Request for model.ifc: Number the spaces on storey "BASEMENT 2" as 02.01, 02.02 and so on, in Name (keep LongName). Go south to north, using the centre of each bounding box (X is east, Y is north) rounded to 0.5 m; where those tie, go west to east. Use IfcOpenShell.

First a look at what the model holds.

```python
import ifcopenshell
import ifcopenshell.util.element
import ifcopenshell.util.placement

model = ifcopenshell.open("model.ifc")
print(model.schema)
storey = next(s for s in model.by_type("IfcBuildingStorey") if s.Name == "BASEMENT 2")
spaces = [e for e in ifcopenshell.util.element.get_decomposition(storey) if e.is_a("IfcSpace")]
for e in sorted(spaces, key=lambda e: e.id()):
    origin = ifcopenshell.util.placement.get_local_placement(e.ObjectPlacement)[:3, 3]
    print(e.id(), e.Name, e.LongName, origin.round(2) + 0.0, sep=" | ")
```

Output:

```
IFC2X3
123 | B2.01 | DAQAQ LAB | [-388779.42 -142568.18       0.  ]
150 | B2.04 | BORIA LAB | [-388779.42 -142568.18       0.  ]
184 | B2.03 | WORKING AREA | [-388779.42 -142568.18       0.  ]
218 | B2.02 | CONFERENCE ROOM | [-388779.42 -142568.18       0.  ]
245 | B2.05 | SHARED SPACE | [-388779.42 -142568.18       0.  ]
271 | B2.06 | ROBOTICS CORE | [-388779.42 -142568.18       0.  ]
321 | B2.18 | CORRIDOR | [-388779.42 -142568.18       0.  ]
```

```python
import ifcopenshell
import ifcopenshell.geom
import ifcopenshell.util.element
import ifcopenshell.util.shape

model = ifcopenshell.open("model.ifc")
settings = ifcopenshell.geom.settings()
settings.set("use-world-coords", True)


def centre(element):
    shape = ifcopenshell.geom.create_shape(settings, element)
    return ifcopenshell.util.shape.get_bbox_centroid(shape.geometry)


storey = next(s for s in model.by_type("IfcBuildingStorey") if s.Name == "BASEMENT 2")
spaces = [e for e in ifcopenshell.util.element.get_decomposition(storey) if e.is_a("IfcSpace")]

# Insertion points can sit at a corner or the storey origin, so sort by the geometry (in metres).
centres = {e: centre(e) for e in spaces}
spaces.sort(key=lambda e: (round(centres[e][1] / 0.5), centres[e][0]))

for i, e in enumerate(spaces, start=1):
    number = f"02.{i:02d}"
    e.Name = number
    print(e.id(), number)

model.write("model-out.ifc")
```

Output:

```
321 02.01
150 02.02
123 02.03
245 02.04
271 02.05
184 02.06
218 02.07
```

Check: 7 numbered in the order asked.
